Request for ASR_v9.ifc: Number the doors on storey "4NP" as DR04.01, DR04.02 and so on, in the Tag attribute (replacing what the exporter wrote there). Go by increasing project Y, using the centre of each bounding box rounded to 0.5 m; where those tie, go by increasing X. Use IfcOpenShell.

First a look at what the model holds.

```python
import ifcopenshell
import ifcopenshell.util.element
import ifcopenshell.util.placement

model = ifcopenshell.open("ASR_v9.ifc")
print(model.schema)
storey = next(s for s in model.by_type("IfcBuildingStorey") if s.Name == "4NP")
doors = [e for e in ifcopenshell.util.element.get_decomposition(storey) if e.is_a("IfcDoor")]
for e in sorted(doors, key=lambda e: e.id()):
    origin = ifcopenshell.util.placement.get_local_placement(e.ObjectPlacement)[:3, 3]
    print(e.id(), e.Tag, e.Name, origin.round(2) + 0.0, sep=" | ")
```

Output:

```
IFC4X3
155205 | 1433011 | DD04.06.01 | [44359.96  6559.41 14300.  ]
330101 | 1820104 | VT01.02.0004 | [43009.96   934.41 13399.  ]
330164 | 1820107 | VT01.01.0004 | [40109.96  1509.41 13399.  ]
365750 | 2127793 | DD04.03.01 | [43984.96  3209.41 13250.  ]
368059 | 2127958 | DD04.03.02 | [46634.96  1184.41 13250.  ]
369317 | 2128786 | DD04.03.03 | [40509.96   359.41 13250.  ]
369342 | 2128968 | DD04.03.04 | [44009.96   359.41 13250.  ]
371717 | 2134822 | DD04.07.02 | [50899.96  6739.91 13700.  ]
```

```python
import ifcopenshell
import ifcopenshell.geom
import ifcopenshell.util.element
import ifcopenshell.util.shape

model = ifcopenshell.open("ASR_v9.ifc")
settings = ifcopenshell.geom.settings()
settings.set("use-world-coords", True)


def centre(element):
    shape = ifcopenshell.geom.create_shape(settings, element)
    return ifcopenshell.util.shape.get_bbox_centroid(shape.geometry)


storey = next(s for s in model.by_type("IfcBuildingStorey") if s.Name == "4NP")
doors = [e for e in ifcopenshell.util.element.get_decomposition(storey) if e.is_a("IfcDoor")]

# Insertion points can sit at a corner or the storey origin, so sort by the geometry (in metres).
centres = {e: centre(e) for e in doors}
doors.sort(key=lambda e: (round(centres[e][1] / 0.5), centres[e][0]))

for i, e in enumerate(doors, start=1):
    number = f"DR04.{i:02d}"
    e.Tag = number
    print(e.id(), number)

model.write("ASR_v9-out.ifc")
```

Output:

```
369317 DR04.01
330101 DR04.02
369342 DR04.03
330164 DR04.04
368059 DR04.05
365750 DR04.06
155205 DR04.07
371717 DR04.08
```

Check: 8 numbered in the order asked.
